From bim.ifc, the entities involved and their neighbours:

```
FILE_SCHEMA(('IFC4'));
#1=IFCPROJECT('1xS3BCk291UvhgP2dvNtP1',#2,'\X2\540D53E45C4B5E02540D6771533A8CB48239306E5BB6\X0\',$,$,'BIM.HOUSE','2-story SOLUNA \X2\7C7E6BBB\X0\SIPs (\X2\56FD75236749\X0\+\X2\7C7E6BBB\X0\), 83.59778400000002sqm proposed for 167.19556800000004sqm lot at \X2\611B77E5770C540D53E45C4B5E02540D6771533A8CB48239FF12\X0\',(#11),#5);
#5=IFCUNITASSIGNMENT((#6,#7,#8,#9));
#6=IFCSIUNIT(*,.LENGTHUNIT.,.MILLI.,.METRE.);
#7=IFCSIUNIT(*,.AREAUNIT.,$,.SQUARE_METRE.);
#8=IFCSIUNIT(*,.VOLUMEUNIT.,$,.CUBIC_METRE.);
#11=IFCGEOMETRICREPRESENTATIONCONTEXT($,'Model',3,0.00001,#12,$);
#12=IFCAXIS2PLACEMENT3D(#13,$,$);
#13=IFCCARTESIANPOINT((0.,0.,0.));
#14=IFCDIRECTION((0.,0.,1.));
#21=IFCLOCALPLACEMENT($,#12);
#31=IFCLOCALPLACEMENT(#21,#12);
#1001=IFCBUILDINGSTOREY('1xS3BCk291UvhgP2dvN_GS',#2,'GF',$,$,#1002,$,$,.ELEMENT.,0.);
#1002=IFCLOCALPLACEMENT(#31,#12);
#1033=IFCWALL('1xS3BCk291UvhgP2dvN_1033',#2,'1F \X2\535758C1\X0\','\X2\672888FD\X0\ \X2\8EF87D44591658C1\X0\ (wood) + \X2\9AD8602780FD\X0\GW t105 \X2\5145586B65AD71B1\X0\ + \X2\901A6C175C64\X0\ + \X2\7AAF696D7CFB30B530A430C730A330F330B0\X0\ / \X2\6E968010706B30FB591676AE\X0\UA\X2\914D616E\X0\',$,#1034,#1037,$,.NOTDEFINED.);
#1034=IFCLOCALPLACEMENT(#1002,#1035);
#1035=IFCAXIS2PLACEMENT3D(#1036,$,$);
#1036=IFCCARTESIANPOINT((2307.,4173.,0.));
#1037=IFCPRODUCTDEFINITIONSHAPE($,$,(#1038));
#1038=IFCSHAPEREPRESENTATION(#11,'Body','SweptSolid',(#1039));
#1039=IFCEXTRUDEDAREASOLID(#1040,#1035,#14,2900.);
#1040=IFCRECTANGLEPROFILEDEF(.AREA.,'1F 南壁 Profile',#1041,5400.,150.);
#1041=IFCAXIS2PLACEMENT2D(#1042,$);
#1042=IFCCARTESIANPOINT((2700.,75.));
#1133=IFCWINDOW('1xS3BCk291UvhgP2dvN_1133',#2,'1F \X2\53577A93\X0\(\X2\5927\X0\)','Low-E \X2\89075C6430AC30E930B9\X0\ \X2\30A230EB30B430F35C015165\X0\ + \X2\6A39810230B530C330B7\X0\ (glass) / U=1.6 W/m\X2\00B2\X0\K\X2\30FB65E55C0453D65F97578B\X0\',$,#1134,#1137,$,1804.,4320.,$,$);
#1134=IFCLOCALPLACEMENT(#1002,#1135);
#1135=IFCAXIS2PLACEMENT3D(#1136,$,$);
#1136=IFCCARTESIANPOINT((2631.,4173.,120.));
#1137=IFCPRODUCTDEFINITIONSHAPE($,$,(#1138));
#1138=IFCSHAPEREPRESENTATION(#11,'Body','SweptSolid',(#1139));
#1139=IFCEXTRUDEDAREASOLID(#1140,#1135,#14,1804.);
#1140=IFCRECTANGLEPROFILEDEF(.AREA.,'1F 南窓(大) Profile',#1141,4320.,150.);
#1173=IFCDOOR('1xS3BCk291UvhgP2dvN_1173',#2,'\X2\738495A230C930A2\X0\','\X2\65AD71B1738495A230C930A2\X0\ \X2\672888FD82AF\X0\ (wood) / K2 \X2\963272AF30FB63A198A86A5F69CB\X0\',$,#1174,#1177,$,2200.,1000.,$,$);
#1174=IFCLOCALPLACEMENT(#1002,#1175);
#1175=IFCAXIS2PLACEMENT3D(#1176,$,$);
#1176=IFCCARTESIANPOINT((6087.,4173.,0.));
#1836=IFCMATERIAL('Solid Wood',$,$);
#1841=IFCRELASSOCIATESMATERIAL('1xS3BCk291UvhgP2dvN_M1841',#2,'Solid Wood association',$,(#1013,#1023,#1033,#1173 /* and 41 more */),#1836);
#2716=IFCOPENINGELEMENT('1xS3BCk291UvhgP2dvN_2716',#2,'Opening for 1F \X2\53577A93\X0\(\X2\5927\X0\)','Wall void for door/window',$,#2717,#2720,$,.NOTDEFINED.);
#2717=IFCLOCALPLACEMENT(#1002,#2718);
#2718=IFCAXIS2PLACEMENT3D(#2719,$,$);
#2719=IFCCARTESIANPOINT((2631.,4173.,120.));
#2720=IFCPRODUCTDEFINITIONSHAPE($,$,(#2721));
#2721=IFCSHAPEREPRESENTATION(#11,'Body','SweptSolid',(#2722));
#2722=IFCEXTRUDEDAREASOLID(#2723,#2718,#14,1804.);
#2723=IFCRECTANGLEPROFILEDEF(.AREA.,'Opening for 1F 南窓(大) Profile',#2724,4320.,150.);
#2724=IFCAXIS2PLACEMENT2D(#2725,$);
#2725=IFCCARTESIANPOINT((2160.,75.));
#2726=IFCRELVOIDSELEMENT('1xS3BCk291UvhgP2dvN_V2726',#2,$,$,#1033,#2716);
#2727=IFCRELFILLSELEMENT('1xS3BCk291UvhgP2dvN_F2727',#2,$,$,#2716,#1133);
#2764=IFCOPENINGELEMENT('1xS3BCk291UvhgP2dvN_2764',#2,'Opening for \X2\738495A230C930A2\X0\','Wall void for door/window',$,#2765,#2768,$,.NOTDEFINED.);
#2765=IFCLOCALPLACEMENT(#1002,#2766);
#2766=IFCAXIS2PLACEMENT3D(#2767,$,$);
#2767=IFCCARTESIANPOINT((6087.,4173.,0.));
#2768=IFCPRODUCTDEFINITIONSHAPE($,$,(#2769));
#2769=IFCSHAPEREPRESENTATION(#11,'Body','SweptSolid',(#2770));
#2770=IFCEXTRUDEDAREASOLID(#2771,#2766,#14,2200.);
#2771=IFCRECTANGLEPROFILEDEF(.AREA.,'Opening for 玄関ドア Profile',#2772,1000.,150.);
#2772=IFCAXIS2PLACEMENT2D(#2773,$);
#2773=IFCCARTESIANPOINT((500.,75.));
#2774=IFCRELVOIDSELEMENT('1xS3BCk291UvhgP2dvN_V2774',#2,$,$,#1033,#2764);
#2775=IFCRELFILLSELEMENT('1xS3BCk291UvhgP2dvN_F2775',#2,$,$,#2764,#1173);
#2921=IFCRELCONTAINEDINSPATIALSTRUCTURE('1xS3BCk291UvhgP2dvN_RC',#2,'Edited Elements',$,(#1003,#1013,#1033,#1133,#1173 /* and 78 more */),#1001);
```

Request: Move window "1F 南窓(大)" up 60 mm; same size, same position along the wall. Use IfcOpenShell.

```python
import numpy as np
import ifcopenshell
import ifcopenshell.api.geometry
import ifcopenshell.util.placement
import ifcopenshell.util.unit

model = ifcopenshell.open("bim.ifc")
unit_scale = ifcopenshell.util.unit.calculate_unit_scale(model)

window = model.by_guid("1xS3BCk291UvhgP2dvN_1133")
opening = window.FillsVoids[0].RelatingOpeningElement
dz = 0.06 / unit_scale

shift = np.array([0.0, 0.0, dz])
# The window is not placed relative to its opening, so move both.
for product in (opening, window):
    matrix = ifcopenshell.util.placement.get_local_placement(product.ObjectPlacement)
    matrix[:3, 3] += shift
    ifcopenshell.api.geometry.edit_object_placement(model, product=product, matrix=matrix, is_si=False)

print(f"moved by {dz * unit_scale:+.3f} m")

model.write("bim_edited.ifc")
```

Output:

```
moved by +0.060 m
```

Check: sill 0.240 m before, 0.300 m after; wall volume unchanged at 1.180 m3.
